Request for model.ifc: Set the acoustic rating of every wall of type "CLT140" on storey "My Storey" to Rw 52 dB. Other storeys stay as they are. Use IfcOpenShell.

First a look at what the model holds.

```python
import ifcopenshell
import ifcopenshell.util.element

model = ifcopenshell.open("model.ifc")
print(model.schema)
storey = next(s for s in model.by_type("IfcBuildingStorey") if s.Name == "My Storey")
walls = [e for e in ifcopenshell.util.element.get_decomposition(storey) if e.is_a("IfcWall")]
seen = {}
for e in walls:
    element_type = ifcopenshell.util.element.get_type(e)
    key = (element_type.Name if element_type != e and element_type else None, ifcopenshell.util.element.get_pset(e, "Pset_WallCommon", "AcousticRating"))
    seen[key] = seen.get(key, 0) + 1
for (name, value), count in sorted(seen.items(), key=str):
    print(count, "x", name, "|", value)
```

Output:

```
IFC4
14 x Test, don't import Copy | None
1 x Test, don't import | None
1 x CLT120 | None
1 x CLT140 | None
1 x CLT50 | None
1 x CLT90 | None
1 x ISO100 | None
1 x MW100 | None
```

```python
import ifcopenshell
import ifcopenshell.api.pset
import ifcopenshell.util.element

model = ifcopenshell.open("model.ifc")

storey = next(s for s in model.by_type("IfcBuildingStorey") if s.Name == "My Storey")
walls = [e for e in ifcopenshell.util.element.get_decomposition(storey) if e.is_a("IfcWall")]

count = 0
for e in walls:
    element_type = ifcopenshell.util.element.get_type(e)
    if element_type in (None, e) or element_type.Name != "CLT140":
        continue
    # add_pset returns the element's existing set when there is one.
    pset = ifcopenshell.api.pset.add_pset(model, product=e, name="Pset_WallCommon")
    ifcopenshell.api.pset.edit_pset(model, pset=pset, properties={"AcousticRating": "Rw 52 dB"})
    count += 1

print(count, "walls updated")

model.write("model-out.ifc")
```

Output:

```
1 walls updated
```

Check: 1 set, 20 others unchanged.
